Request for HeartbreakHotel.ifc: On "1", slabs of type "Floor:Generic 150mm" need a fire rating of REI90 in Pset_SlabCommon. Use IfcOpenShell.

First a look at what the model holds.

```python
import ifcopenshell
import ifcopenshell.util.element

model = ifcopenshell.open("HeartbreakHotel.ifc")
print(model.schema)
storey = next(s for s in model.by_type("IfcBuildingStorey") if s.Name == "1")
slabs = [e for e in ifcopenshell.util.element.get_decomposition(storey) if e.is_a("IfcSlab")]
seen = {}
for e in slabs:
    element_type = ifcopenshell.util.element.get_type(e)
    key = (element_type.Name if element_type != e and element_type else None, ifcopenshell.util.element.get_pset(e, "Pset_SlabCommon", "FireRating"))
    seen[key] = seen.get(key, 0) + 1
for (name, value), count in sorted(seen.items(), key=str):
    print(count, "x", name, "|", value)
```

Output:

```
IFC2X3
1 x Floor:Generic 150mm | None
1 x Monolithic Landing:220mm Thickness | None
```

```python
import ifcopenshell
import ifcopenshell.api.pset
import ifcopenshell.util.element

model = ifcopenshell.open("HeartbreakHotel.ifc")

storey = next(s for s in model.by_type("IfcBuildingStorey") if s.Name == "1")
slabs = [e for e in ifcopenshell.util.element.get_decomposition(storey) if e.is_a("IfcSlab")]

count = 0
for e in slabs:
    element_type = ifcopenshell.util.element.get_type(e)
    if element_type in (None, e) or element_type.Name != "Floor:Generic 150mm":
        continue
    # add_pset returns the element's existing set when there is one.
    pset = ifcopenshell.api.pset.add_pset(model, product=e, name="Pset_SlabCommon")
    ifcopenshell.api.pset.edit_pset(model, pset=pset, properties={"FireRating": "REI90"})
    count += 1

print(count, "slabs updated")

model.write("HeartbreakHotel_edited.ifc")
```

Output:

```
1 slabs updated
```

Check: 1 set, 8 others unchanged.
